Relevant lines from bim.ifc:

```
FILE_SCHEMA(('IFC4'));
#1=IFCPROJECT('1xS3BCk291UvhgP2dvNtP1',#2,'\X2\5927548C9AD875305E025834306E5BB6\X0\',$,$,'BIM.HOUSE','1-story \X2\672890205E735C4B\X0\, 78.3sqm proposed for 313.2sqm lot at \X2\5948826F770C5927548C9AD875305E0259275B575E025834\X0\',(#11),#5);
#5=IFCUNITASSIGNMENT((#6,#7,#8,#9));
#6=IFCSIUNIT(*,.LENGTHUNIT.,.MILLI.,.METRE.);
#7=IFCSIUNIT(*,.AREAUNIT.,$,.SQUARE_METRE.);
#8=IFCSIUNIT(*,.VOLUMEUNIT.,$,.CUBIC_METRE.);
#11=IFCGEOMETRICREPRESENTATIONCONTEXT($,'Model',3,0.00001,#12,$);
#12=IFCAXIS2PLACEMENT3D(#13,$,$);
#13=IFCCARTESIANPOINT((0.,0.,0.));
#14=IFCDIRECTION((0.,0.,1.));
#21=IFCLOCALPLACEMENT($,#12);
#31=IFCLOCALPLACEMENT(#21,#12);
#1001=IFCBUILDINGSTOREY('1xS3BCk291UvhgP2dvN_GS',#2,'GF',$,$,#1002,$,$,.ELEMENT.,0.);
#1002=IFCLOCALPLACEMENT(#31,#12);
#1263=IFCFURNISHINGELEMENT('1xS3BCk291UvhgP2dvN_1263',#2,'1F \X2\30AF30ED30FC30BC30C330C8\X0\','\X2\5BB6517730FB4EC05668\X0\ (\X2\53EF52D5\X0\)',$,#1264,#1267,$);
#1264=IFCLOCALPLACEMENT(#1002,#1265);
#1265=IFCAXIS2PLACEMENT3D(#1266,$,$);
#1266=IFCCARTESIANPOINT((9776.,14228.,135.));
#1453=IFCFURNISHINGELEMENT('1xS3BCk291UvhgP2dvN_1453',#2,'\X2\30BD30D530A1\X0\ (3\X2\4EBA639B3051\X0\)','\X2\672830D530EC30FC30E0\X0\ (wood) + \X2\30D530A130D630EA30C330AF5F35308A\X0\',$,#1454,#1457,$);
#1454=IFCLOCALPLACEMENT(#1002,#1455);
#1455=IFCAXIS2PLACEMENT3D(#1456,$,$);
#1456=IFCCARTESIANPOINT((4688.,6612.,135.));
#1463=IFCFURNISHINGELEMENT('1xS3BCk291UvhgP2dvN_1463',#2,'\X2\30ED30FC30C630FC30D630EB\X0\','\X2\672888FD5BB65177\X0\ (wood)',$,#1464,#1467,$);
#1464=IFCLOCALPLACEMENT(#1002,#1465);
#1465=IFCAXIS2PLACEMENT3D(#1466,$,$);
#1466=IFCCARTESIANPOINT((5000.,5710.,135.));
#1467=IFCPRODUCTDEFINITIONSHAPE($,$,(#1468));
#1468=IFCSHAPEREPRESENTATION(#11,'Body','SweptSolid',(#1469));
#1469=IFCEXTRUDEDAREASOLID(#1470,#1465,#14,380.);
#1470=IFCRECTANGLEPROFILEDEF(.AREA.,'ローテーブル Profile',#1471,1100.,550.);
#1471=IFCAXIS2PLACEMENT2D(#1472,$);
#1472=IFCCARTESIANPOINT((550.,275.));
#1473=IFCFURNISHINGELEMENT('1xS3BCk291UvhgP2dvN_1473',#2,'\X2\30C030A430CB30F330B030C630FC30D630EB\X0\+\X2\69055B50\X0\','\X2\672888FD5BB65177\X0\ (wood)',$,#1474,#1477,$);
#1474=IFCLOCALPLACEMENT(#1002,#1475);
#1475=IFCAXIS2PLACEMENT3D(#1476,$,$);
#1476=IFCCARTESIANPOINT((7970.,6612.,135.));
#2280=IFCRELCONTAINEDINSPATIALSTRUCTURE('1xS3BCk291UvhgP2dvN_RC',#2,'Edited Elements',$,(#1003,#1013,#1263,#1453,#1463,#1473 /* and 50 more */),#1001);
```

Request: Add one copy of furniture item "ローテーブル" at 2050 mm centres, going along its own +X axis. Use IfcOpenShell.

```python
import ifcopenshell
import ifcopenshell.api.geometry
import ifcopenshell.api.root
import ifcopenshell.util.element
import ifcopenshell.util.placement
import ifcopenshell.util.unit

model = ifcopenshell.open("bim.ifc")
unit_scale = ifcopenshell.util.unit.calculate_unit_scale(model)


def reuse_history(source, copy):
    """copy_class also copies each property set's owner history, people and application; keep the originals."""
    for rel in copy.IsDefinedBy:
        if rel.is_a("IfcRelDefinesByProperties") and (history := rel.RelatingPropertyDefinition.OwnerHistory):
            rel.RelatingPropertyDefinition.OwnerHistory = source.OwnerHistory
            ifcopenshell.util.element.remove_deep2(model, history)


source = model.by_id(1463)
base = ifcopenshell.util.placement.get_local_placement(source.ObjectPlacement)
step = base[:3, 0] * 2.05 / unit_scale

for i in range(1, 2):
    copy = ifcopenshell.api.root.copy_class(model, product=source)
    copy.Representation = ifcopenshell.util.element.copy_deep(
        model, source.Representation, exclude=["IfcGeometricRepresentationContext", "IfcRepresentationMap"]
    )
    reuse_history(source, copy)
    matrix = base.copy()
    matrix[:3, 3] += i * step
    print("added at", matrix[:3, 3].round(3) + 0.0)
    ifcopenshell.api.geometry.edit_object_placement(model, product=copy, matrix=matrix, is_si=False)

model.write("bim-out.ifc")
```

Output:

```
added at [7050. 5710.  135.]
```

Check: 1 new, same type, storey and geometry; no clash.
